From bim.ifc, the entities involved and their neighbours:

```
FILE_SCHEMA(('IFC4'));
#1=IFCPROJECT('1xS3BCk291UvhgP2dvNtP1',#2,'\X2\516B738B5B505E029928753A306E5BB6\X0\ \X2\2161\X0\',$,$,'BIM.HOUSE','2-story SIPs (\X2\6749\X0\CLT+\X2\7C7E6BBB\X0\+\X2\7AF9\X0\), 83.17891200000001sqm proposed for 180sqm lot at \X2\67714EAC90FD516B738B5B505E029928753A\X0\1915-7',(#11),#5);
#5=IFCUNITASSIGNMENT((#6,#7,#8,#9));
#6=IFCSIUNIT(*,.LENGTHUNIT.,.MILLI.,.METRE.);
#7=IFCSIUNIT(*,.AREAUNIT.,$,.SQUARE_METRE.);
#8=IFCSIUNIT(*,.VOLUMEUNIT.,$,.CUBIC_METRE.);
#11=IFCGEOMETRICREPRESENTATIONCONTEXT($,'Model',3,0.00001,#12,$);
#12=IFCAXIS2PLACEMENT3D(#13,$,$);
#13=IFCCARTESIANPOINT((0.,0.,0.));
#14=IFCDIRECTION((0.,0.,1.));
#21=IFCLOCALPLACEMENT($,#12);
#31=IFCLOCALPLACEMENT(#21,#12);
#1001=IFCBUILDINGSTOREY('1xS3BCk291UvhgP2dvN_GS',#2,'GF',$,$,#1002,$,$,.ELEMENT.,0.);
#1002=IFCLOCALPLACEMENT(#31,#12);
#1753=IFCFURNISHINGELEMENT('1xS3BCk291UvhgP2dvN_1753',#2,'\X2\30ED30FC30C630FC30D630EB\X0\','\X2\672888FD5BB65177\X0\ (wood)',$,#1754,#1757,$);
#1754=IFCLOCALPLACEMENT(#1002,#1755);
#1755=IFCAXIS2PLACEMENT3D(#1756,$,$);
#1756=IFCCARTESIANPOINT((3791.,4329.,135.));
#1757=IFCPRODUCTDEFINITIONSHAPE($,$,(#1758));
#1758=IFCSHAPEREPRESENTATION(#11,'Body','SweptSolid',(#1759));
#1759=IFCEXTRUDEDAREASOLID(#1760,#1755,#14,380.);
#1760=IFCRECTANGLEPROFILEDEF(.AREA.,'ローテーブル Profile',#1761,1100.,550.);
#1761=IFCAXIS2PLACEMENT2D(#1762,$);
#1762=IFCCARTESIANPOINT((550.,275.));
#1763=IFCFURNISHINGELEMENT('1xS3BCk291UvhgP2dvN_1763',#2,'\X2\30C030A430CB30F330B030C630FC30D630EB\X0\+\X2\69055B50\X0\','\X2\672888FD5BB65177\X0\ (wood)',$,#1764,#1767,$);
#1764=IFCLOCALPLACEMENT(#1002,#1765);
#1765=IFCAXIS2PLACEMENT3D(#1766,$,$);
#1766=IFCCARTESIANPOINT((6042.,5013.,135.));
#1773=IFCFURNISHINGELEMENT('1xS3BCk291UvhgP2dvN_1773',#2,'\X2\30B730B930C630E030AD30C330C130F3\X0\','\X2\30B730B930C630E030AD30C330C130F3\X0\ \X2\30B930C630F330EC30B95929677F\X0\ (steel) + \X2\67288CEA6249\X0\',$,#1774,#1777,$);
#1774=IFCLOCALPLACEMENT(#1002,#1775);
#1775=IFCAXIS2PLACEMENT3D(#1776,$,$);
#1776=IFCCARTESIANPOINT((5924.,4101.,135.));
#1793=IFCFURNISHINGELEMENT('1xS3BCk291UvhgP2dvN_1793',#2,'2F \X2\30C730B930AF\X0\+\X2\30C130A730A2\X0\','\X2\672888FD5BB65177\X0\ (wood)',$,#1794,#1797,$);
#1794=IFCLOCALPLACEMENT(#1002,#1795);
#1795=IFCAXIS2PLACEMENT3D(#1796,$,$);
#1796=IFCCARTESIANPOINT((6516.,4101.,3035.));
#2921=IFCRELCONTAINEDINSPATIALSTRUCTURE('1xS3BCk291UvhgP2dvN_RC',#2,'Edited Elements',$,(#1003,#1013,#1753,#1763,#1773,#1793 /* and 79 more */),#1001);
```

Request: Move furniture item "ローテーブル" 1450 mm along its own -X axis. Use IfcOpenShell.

```python
import ifcopenshell
import ifcopenshell.api.geometry
import ifcopenshell.util.placement

model = ifcopenshell.open("bim.ifc")

item = model.by_id(1753)
matrix = ifcopenshell.util.placement.get_local_placement(item.ObjectPlacement)
matrix[:3, 3] -= matrix[:3, 0] * 1450.0
ifcopenshell.api.geometry.edit_object_placement(model, product=item, matrix=matrix, is_si=False)

print(ifcopenshell.util.placement.get_local_placement(item.ObjectPlacement).round(3) + 0.0)

model.write("bim_updated.ifc")
```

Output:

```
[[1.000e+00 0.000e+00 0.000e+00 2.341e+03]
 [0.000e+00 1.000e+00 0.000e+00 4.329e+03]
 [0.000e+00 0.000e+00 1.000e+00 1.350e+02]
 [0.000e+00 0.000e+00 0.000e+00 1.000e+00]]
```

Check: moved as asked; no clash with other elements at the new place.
